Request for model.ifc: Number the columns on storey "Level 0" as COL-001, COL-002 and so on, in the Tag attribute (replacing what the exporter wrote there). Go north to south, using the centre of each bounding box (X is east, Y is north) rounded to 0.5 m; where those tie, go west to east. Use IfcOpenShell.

First a look at what the model holds.

```python
import ifcopenshell
import ifcopenshell.util.element
import ifcopenshell.util.placement

model = ifcopenshell.open("model.ifc")
print(model.schema)
storey = next(s for s in model.by_type("IfcBuildingStorey") if s.Name == "Level 0")
columns = [e for e in ifcopenshell.util.element.get_decomposition(storey) if e.is_a("IfcColumn")]
for e in sorted(columns, key=lambda e: e.id()):
    origin = ifcopenshell.util.placement.get_local_placement(e.ObjectPlacement)[:3, 3]
    print(e.id(), e.Tag, e.Name, origin.round(2) + 0.0, sep=" | ")
```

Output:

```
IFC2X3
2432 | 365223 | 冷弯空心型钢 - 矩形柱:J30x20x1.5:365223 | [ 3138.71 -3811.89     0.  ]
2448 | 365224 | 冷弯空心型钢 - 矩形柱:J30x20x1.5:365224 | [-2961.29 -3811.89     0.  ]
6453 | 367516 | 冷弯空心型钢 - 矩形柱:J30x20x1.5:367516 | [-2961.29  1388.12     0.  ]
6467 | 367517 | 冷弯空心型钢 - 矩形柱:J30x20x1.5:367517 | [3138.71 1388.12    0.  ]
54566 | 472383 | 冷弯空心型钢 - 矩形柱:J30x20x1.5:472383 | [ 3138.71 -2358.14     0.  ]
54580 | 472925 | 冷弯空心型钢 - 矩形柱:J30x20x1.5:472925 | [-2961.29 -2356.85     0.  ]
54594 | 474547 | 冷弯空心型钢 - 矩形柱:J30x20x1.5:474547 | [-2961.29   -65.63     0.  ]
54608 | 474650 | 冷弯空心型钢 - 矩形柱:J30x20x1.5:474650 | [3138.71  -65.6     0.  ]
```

```python
import ifcopenshell
import ifcopenshell.geom
import ifcopenshell.util.element
import ifcopenshell.util.shape

model = ifcopenshell.open("model.ifc")
settings = ifcopenshell.geom.settings()
settings.set("use-world-coords", True)


def centre(element):
    shape = ifcopenshell.geom.create_shape(settings, element)
    return ifcopenshell.util.shape.get_bbox_centroid(shape.geometry)


storey = next(s for s in model.by_type("IfcBuildingStorey") if s.Name == "Level 0")
columns = [e for e in ifcopenshell.util.element.get_decomposition(storey) if e.is_a("IfcColumn")]

# Insertion points can sit at a corner or the storey origin, so sort by the geometry (in metres).
centres = {e: centre(e) for e in columns}
columns.sort(key=lambda e: (-round(centres[e][1] / 0.5), centres[e][0]))

for i, e in enumerate(columns, start=1):
    number = f"COL-0{i:02d}"
    e.Tag = number
    print(e.id(), number)

model.write("model_edited.ifc")
```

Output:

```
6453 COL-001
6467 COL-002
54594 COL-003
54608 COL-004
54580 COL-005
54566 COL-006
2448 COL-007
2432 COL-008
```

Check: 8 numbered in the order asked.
